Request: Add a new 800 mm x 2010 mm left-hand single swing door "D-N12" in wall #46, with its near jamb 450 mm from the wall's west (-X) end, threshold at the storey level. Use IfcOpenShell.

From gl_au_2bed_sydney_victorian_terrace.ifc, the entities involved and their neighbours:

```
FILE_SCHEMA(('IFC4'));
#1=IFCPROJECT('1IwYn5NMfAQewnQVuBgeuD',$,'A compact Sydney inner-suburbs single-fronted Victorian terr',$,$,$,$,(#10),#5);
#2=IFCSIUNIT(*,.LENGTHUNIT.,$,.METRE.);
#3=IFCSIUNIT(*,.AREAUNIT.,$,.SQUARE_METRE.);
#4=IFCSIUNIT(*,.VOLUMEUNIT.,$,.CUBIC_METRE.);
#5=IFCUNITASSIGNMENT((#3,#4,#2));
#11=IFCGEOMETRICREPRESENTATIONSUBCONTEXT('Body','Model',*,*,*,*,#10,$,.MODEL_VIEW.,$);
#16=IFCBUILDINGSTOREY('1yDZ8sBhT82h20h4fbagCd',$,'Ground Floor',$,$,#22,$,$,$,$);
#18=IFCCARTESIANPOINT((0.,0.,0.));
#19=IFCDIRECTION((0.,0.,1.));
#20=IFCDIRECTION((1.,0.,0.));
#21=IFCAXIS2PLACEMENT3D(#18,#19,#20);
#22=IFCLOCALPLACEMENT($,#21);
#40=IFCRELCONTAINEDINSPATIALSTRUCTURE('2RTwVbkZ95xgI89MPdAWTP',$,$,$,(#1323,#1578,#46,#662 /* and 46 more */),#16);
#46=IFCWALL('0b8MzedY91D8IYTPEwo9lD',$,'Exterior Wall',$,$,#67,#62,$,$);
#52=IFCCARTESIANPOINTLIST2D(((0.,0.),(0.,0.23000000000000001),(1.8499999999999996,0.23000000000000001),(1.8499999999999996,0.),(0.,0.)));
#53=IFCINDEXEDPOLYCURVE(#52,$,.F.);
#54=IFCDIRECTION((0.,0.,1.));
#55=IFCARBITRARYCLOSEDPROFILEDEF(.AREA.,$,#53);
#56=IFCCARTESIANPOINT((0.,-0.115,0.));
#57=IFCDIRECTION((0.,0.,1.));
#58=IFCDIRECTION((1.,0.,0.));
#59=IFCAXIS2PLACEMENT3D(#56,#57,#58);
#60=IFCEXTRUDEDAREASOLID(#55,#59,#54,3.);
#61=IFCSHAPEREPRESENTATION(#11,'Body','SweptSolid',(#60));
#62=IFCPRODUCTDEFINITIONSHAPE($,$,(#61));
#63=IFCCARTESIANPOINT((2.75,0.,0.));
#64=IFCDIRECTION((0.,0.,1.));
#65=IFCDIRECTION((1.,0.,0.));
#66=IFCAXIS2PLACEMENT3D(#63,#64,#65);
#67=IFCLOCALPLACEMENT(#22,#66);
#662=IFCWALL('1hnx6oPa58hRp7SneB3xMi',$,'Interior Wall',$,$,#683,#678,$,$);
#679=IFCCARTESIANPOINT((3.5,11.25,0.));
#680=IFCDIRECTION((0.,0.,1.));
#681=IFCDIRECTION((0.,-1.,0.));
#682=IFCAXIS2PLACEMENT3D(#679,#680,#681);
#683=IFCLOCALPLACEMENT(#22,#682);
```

```python
import numpy as np
import ifcopenshell
import ifcopenshell.api.feature
import ifcopenshell.api.geometry
import ifcopenshell.api.root
import ifcopenshell.api.spatial
import ifcopenshell.geom
import ifcopenshell.util.element
import ifcopenshell.util.placement
import ifcopenshell.util.representation
import ifcopenshell.util.shape
import ifcopenshell.util.unit

model = ifcopenshell.open("gl_au_2bed_sydney_victorian_terrace.ifc")
unit_scale = ifcopenshell.util.unit.calculate_unit_scale(model)
settings = ifcopenshell.geom.settings()


def volume(element):
    """Net volume in cubic metres, openings subtracted."""
    shape = ifcopenshell.geom.create_shape(settings, element)
    return ifcopenshell.util.shape.get_volume(shape.geometry)


wall = model.by_guid("0b8MzedY91D8IYTPEwo9lD")
storey = ifcopenshell.util.element.get_container(wall, ifc_class="IfcBuildingStorey")
context = ifcopenshell.util.representation.get_context(model, "Model", "Body", "MODEL_VIEW")
before = volume(wall)

width, height, from_end, sill = 0.8, 2.01, 0.45, 0.0  # metres

# The wall runs along its own X axis, and the end named is its -X end.
wall_shape = ifcopenshell.geom.create_shape(settings, wall)
x, y, z = ifcopenshell.util.shape.get_vertices(wall_shape.geometry).T
start = x.min() + from_end
face, thickness = float(y.min()), float(y.max() - y.min())
wall_matrix = ifcopenshell.util.placement.get_local_placement(wall.ObjectPlacement)
level = ifcopenshell.util.placement.get_local_placement(storey.ObjectPlacement)[2, 3]


def in_wall(x, y):
    """Placement at x, y metres in the wall's axes, at sill height."""
    matrix = wall_matrix.copy()
    matrix[:, 3] = wall_matrix @ np.array([x / unit_scale, y / unit_scale, 0.0, 1.0])
    matrix[2, 3] = level + sill / unit_scale
    return matrix


# Opening: a box that overshoots both wall faces by 50 mm.
opening = ifcopenshell.api.root.create_entity(model, ifc_class="IfcOpeningElement", predefined_type="OPENING")
box = ifcopenshell.api.geometry.add_wall_representation(
    model, context=context, length=width, height=height, thickness=thickness + 0.1
)
ifcopenshell.api.geometry.assign_representation(model, product=opening, representation=box)
ifcopenshell.api.geometry.edit_object_placement(model, product=opening, matrix=in_wall(start, face - 0.05), is_si=False)
ifcopenshell.api.feature.add_feature(model, feature=opening, element=wall)

door = ifcopenshell.api.root.create_entity(model, ifc_class="IfcDoor", name="D-N12", predefined_type="DOOR")
door.OverallWidth, door.OverallHeight = width / unit_scale, height / unit_scale
door.OperationType = "SINGLE_SWING_LEFT"
body = ifcopenshell.api.geometry.add_door_representation(
    model,
    context=context,
    overall_width=door.OverallWidth,
    overall_height=door.OverallHeight,
    operation_type="SINGLE_SWING_LEFT",
    lining_properties={"LiningDepth": thickness / unit_scale, "ThresholdDepth": thickness / unit_scale},
)
ifcopenshell.api.geometry.assign_representation(model, product=door, representation=body)
ifcopenshell.api.spatial.assign_container(model, products=[door], relating_structure=storey)
ifcopenshell.api.feature.add_filling(model, opening=opening, element=door)

# The lining spans the wall, so the door starts at the wall face.
ifcopenshell.api.geometry.edit_object_placement(model, product=door, matrix=in_wall(start, face), is_si=False)

after = volume(wall)

print(f"wall volume {before:.3f} -> {after:.3f} m3")

model.write("gl_au_2bed_sydney_victorian_terrace_updated.ifc")
```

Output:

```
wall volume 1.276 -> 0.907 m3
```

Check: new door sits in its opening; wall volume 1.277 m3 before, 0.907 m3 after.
